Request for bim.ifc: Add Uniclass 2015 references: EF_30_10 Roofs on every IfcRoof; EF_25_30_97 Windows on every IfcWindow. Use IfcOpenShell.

First a look at what the model holds.

```python
import ifcopenshell

model = ifcopenshell.open("bim.ifc")
print(model.schema)
print("classifications:", [c.Name for c in model.by_type("IfcClassification")])
for ifc_class in ("IfcDoor", "IfcRoof", "IfcStair", "IfcWall", "IfcWindow"):
    print(ifc_class, len(model.by_type(ifc_class)))
```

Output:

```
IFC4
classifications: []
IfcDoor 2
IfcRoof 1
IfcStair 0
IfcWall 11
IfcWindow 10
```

```python
import ifcopenshell
import ifcopenshell.api.classification

model = ifcopenshell.open("bim.ifc")

system = ifcopenshell.api.classification.add_classification(model, classification="Uniclass 2015")

codes = {
    "IfcRoof": ("EF_30_10", "Roofs"),
    "IfcWindow": ("EF_25_30_97", "Windows"),
}
for ifc_class, (code, name) in codes.items():
    products = model.by_type(ifc_class)
    ifcopenshell.api.classification.add_reference(
        model, products=products, classification=system, identification=code, name=name
    )
    print(code, len(products))

model.write("bim_v2.ifc")
```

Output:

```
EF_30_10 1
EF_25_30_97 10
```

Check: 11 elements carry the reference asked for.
